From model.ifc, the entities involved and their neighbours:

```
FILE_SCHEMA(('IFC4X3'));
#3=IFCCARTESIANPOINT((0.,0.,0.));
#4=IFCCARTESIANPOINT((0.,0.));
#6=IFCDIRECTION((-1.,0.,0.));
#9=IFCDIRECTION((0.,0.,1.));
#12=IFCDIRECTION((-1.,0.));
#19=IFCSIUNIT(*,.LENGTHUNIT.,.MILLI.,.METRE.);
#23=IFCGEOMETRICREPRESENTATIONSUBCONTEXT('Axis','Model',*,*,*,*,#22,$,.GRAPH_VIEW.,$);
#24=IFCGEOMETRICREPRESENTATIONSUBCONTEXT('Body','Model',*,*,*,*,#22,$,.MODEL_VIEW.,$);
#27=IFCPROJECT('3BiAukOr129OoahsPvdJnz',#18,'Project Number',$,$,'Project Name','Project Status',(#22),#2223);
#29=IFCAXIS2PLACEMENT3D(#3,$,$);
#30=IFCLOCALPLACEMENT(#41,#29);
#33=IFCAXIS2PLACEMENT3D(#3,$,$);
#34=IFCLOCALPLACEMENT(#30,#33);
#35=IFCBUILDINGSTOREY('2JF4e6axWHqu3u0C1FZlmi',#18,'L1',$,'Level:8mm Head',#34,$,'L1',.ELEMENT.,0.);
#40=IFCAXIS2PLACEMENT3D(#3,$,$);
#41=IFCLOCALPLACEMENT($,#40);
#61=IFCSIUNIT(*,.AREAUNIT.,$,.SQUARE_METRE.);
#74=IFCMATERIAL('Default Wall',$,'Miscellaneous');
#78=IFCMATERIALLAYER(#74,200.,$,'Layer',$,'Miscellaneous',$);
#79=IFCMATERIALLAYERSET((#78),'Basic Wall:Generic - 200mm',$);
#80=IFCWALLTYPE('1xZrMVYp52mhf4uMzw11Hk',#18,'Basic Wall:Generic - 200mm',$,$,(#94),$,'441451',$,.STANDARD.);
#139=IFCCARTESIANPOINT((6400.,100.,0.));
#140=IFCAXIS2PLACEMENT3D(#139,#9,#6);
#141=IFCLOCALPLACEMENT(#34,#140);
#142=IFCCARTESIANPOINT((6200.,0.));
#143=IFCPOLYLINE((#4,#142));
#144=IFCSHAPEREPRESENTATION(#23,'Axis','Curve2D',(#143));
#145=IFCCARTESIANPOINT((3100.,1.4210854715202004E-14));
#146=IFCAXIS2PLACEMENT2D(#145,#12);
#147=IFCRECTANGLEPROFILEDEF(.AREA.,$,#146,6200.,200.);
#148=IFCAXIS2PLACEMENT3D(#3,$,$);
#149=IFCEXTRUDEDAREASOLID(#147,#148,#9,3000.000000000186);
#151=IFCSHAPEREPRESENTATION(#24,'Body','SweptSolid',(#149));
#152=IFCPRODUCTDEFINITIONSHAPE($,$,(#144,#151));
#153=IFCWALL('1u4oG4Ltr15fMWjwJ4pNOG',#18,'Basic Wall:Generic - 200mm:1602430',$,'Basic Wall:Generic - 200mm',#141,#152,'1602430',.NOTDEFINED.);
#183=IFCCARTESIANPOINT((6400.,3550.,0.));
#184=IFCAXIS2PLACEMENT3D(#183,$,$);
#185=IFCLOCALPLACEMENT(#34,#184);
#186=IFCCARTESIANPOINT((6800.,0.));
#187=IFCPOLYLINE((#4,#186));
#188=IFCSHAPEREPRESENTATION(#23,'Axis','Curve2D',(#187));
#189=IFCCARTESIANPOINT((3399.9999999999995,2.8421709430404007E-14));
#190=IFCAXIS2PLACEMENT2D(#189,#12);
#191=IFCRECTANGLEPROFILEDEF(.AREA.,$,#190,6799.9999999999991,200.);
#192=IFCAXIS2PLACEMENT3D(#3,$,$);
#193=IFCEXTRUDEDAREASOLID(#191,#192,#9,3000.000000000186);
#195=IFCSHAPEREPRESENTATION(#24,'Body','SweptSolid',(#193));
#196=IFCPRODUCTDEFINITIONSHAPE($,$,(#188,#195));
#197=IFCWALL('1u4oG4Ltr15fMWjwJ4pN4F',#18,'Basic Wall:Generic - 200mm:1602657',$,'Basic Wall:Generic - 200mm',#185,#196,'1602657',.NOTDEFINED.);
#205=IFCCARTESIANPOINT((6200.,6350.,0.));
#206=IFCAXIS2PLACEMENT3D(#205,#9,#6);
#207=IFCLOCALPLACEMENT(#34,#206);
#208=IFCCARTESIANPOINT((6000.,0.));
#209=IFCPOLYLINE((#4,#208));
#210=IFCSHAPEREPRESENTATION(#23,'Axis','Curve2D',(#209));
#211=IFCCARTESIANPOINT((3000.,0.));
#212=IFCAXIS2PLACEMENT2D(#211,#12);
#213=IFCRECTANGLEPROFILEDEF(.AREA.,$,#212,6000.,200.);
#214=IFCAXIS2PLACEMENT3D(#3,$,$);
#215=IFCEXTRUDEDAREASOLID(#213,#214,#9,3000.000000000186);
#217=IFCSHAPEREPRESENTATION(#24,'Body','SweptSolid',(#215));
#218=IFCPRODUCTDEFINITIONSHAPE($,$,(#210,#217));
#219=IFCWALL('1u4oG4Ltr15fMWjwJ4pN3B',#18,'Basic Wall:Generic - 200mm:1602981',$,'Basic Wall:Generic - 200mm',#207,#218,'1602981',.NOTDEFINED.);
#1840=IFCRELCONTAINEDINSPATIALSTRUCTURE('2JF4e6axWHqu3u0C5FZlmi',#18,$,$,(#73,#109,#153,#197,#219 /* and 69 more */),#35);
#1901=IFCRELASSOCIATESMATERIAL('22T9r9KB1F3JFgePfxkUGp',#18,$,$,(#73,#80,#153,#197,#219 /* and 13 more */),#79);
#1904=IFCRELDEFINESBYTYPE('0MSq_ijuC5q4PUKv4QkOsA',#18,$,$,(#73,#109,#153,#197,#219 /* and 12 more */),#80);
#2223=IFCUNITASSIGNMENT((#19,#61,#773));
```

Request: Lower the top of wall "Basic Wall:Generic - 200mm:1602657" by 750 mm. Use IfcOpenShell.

```python
import ifcopenshell
import ifcopenshell.geom
import ifcopenshell.util.representation
import ifcopenshell.util.shape

model = ifcopenshell.open("model.ifc")
settings = ifcopenshell.geom.settings()


def volume(element):
    """Net volume in cubic metres, openings subtracted."""
    shape = ifcopenshell.geom.create_shape(settings, element)
    return ifcopenshell.util.shape.get_volume(shape.geometry)


wall = model.by_guid("1u4oG4Ltr15fMWjwJ4pN4F")
before = volume(wall)

body = ifcopenshell.util.representation.get_representation(wall, "Model", "Body")
solid = body.Items[0]
old_height = solid.Depth
solid.Depth -= 750.0
after = volume(wall)

print(f"height {old_height:g} -> {solid.Depth:g}, volume {before:.3f} -> {after:.3f} m3")

model.write("model_v2.ifc")
```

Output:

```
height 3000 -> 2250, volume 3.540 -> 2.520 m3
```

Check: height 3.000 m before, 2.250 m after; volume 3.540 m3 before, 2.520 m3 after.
